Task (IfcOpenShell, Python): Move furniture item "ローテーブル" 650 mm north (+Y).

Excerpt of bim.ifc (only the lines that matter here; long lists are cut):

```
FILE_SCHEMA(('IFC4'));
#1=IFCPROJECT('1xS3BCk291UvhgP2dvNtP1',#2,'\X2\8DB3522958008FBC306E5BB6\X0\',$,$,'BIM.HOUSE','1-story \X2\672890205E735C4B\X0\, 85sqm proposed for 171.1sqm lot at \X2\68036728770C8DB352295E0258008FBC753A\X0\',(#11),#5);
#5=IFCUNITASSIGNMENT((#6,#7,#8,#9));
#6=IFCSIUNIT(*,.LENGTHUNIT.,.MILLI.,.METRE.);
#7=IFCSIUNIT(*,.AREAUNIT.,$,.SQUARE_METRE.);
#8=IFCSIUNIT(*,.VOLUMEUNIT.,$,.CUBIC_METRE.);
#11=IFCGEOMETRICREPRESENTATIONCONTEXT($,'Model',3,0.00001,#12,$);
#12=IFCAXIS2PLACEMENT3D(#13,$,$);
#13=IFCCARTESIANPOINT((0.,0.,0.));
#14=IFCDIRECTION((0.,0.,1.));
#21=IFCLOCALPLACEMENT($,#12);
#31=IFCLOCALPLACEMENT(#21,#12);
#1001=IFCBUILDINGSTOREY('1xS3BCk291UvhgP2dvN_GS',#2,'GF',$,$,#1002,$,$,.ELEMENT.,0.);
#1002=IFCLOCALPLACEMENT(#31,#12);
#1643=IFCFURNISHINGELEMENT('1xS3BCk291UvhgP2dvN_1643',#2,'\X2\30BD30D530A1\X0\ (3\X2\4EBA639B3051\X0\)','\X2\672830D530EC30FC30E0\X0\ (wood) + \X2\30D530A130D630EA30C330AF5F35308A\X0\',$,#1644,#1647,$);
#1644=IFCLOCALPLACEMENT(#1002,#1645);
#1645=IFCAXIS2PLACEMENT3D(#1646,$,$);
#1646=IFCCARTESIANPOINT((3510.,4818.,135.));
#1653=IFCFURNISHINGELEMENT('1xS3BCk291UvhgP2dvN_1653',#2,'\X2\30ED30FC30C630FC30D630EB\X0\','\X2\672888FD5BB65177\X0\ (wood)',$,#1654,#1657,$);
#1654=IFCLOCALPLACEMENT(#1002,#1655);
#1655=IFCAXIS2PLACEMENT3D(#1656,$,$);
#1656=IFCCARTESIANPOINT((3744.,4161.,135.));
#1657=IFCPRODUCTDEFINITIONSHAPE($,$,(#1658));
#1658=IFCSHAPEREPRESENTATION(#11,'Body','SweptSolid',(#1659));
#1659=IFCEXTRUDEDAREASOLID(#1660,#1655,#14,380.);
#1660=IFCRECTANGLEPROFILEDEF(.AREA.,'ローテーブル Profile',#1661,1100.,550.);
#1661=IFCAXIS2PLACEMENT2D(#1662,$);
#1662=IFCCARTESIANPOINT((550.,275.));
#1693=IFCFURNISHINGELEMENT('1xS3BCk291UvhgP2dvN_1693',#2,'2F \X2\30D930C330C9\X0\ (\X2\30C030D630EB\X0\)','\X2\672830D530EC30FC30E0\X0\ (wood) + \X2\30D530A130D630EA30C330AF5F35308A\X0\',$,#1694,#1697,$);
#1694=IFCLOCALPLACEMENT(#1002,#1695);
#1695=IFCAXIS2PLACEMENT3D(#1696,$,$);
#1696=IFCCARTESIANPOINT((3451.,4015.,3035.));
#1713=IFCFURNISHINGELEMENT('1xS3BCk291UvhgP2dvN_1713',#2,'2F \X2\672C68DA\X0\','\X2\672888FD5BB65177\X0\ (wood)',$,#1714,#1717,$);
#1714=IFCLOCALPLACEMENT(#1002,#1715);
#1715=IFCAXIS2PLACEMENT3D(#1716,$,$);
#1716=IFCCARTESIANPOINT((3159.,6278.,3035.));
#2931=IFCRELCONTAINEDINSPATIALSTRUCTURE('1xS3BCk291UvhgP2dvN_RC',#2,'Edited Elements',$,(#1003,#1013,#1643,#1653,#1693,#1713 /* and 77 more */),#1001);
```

```python
import ifcopenshell
import ifcopenshell.api.geometry
import ifcopenshell.util.placement

model = ifcopenshell.open("bim.ifc")

item = model.by_id(1653)
matrix = ifcopenshell.util.placement.get_local_placement(item.ObjectPlacement)
matrix[1, 3] += 650.0
ifcopenshell.api.geometry.edit_object_placement(model, product=item, matrix=matrix, is_si=False)

print(ifcopenshell.util.placement.get_local_placement(item.ObjectPlacement).round(3) + 0.0)

model.write("bim_edited.ifc")
```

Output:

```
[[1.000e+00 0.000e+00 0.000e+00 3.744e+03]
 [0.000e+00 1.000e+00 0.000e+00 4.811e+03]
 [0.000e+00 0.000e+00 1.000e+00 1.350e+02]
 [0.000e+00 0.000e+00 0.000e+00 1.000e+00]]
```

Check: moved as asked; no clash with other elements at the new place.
